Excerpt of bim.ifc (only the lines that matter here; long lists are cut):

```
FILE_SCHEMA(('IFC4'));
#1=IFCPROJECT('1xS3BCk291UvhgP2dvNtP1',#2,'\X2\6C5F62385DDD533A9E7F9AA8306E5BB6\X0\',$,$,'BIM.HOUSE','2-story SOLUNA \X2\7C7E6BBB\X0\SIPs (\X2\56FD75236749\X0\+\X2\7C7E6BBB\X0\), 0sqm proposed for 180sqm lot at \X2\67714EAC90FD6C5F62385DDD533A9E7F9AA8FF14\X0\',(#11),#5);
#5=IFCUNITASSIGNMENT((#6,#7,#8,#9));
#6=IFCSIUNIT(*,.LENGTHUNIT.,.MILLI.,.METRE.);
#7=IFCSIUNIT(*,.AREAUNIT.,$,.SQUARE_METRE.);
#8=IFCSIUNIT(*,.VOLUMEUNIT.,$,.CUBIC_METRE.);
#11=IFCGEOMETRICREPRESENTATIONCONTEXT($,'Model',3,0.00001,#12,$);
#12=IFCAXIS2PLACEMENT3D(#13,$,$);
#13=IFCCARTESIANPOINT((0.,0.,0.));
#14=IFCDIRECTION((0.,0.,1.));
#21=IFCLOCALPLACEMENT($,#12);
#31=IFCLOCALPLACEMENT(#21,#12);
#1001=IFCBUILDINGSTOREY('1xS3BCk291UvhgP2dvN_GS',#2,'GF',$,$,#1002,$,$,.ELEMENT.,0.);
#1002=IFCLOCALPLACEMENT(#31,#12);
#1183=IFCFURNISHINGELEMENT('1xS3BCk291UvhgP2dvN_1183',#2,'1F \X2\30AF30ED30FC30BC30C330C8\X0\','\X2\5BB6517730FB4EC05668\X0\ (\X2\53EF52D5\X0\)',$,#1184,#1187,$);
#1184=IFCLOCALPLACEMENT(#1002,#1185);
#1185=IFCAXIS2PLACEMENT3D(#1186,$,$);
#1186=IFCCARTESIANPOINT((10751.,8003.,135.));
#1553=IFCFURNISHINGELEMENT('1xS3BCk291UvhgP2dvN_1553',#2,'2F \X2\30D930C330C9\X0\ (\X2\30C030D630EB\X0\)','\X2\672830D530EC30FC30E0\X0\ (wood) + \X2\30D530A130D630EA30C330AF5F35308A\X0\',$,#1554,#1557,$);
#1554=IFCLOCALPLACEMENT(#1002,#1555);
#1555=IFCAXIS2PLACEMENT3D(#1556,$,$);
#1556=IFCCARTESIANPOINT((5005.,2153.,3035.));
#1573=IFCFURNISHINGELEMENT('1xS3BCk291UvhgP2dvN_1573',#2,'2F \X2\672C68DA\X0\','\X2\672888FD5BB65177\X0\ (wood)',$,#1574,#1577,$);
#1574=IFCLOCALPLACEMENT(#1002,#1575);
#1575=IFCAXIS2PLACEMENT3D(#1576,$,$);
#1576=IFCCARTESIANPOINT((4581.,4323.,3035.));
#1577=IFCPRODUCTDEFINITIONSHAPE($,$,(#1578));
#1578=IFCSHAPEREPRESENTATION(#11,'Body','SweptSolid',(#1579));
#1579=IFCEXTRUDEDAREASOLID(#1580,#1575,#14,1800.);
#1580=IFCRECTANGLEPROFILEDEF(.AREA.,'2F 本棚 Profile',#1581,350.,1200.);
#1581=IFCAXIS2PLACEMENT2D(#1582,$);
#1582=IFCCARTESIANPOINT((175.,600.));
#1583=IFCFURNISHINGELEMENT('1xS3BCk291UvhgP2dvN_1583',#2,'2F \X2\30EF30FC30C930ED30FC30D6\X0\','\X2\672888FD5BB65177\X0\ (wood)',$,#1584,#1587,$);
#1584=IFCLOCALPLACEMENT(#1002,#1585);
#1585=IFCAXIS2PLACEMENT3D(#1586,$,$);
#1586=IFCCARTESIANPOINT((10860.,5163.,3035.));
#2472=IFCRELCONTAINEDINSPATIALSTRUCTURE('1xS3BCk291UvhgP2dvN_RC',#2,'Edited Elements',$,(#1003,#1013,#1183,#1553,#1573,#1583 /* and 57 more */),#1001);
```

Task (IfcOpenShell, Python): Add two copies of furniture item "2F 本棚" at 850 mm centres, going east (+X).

```python
import numpy as np
import ifcopenshell
import ifcopenshell.api.geometry
import ifcopenshell.api.root
import ifcopenshell.util.element
import ifcopenshell.util.placement

model = ifcopenshell.open("bim.ifc")


def reuse_history(source, copy):
    """copy_class also copies each property set's owner history, people and application; keep the originals."""
    for rel in copy.IsDefinedBy:
        if rel.is_a("IfcRelDefinesByProperties") and (history := rel.RelatingPropertyDefinition.OwnerHistory):
            rel.RelatingPropertyDefinition.OwnerHistory = source.OwnerHistory
            ifcopenshell.util.element.remove_deep2(model, history)


source = model.by_guid("1xS3BCk291UvhgP2dvN_1573")
base = ifcopenshell.util.placement.get_local_placement(source.ObjectPlacement)
step = np.array([1.0, 0.0, 0.0]) * 850.0

for i in range(1, 3):
    copy = ifcopenshell.api.root.copy_class(model, product=source)
    copy.Representation = ifcopenshell.util.element.copy_deep(
        model, source.Representation, exclude=["IfcGeometricRepresentationContext", "IfcRepresentationMap"]
    )
    reuse_history(source, copy)
    matrix = base.copy()
    matrix[:3, 3] += i * step
    print("added at", matrix[:3, 3].round(3) + 0.0)
    ifcopenshell.api.geometry.edit_object_placement(model, product=copy, matrix=matrix, is_si=False)

model.write("bim_rev.ifc")
```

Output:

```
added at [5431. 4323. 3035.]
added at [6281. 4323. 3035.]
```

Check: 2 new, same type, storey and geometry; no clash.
